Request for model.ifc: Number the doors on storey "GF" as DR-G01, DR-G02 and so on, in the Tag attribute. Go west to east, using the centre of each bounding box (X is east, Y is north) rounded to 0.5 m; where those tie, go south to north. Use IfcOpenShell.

First a look at what the model holds.

```python
import ifcopenshell
import ifcopenshell.util.element
import ifcopenshell.util.placement

model = ifcopenshell.open("model.ifc")
print(model.schema)
storey = next(s for s in model.by_type("IfcBuildingStorey") if s.Name == "GF")
doors = [e for e in ifcopenshell.util.element.get_decomposition(storey) if e.is_a("IfcDoor")]
for e in sorted(doors, key=lambda e: e.id()):
    origin = ifcopenshell.util.placement.get_local_placement(e.ObjectPlacement)[:3, 3]
    print(e.id(), e.Tag, e.Name, origin.round(2) + 0.0, sep=" | ")
```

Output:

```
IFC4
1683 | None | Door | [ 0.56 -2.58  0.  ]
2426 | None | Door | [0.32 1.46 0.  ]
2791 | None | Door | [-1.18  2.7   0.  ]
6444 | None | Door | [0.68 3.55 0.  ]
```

```python
import ifcopenshell
import ifcopenshell.geom
import ifcopenshell.util.element
import ifcopenshell.util.shape

model = ifcopenshell.open("model.ifc")
settings = ifcopenshell.geom.settings()
settings.set("use-world-coords", True)


def centre(element):
    shape = ifcopenshell.geom.create_shape(settings, element)
    return ifcopenshell.util.shape.get_bbox_centroid(shape.geometry)


storey = next(s for s in model.by_type("IfcBuildingStorey") if s.Name == "GF")
doors = [e for e in ifcopenshell.util.element.get_decomposition(storey) if e.is_a("IfcDoor")]

# Insertion points can sit at a corner or the storey origin, so sort by the geometry (in metres).
centres = {e: centre(e) for e in doors}
doors.sort(key=lambda e: (round(centres[e][0] / 0.5), centres[e][1]))

for i, e in enumerate(doors, start=1):
    number = f"DR-G{i:02d}"
    e.Tag = number
    print(e.id(), number)

model.write("model_v2.ifc")
```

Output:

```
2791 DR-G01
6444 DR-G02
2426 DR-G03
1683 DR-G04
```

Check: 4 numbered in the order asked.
